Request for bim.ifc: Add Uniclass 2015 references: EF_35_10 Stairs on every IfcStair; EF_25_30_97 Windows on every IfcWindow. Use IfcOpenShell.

First a look at what the model holds.

```python
import ifcopenshell

model = ifcopenshell.open("bim.ifc")
print(model.schema)
print("classifications:", [c.Name for c in model.by_type("IfcClassification")])
for ifc_class in ("IfcDoor", "IfcRoof", "IfcStair", "IfcWall", "IfcWindow"):
    print(ifc_class, len(model.by_type(ifc_class)))
```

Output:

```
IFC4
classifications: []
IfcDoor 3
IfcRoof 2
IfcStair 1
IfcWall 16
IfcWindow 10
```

```python
import ifcopenshell
import ifcopenshell.api.classification

model = ifcopenshell.open("bim.ifc")

system = ifcopenshell.api.classification.add_classification(model, classification="Uniclass 2015")

codes = {
    "IfcStair": ("EF_35_10", "Stairs"),
    "IfcWindow": ("EF_25_30_97", "Windows"),
}
for ifc_class, (code, name) in codes.items():
    products = model.by_type(ifc_class)
    ifcopenshell.api.classification.add_reference(
        model, products=products, classification=system, identification=code, name=name
    )
    print(code, len(products))

model.write("bim_v2.ifc")
```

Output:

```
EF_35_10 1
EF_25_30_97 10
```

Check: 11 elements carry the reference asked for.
